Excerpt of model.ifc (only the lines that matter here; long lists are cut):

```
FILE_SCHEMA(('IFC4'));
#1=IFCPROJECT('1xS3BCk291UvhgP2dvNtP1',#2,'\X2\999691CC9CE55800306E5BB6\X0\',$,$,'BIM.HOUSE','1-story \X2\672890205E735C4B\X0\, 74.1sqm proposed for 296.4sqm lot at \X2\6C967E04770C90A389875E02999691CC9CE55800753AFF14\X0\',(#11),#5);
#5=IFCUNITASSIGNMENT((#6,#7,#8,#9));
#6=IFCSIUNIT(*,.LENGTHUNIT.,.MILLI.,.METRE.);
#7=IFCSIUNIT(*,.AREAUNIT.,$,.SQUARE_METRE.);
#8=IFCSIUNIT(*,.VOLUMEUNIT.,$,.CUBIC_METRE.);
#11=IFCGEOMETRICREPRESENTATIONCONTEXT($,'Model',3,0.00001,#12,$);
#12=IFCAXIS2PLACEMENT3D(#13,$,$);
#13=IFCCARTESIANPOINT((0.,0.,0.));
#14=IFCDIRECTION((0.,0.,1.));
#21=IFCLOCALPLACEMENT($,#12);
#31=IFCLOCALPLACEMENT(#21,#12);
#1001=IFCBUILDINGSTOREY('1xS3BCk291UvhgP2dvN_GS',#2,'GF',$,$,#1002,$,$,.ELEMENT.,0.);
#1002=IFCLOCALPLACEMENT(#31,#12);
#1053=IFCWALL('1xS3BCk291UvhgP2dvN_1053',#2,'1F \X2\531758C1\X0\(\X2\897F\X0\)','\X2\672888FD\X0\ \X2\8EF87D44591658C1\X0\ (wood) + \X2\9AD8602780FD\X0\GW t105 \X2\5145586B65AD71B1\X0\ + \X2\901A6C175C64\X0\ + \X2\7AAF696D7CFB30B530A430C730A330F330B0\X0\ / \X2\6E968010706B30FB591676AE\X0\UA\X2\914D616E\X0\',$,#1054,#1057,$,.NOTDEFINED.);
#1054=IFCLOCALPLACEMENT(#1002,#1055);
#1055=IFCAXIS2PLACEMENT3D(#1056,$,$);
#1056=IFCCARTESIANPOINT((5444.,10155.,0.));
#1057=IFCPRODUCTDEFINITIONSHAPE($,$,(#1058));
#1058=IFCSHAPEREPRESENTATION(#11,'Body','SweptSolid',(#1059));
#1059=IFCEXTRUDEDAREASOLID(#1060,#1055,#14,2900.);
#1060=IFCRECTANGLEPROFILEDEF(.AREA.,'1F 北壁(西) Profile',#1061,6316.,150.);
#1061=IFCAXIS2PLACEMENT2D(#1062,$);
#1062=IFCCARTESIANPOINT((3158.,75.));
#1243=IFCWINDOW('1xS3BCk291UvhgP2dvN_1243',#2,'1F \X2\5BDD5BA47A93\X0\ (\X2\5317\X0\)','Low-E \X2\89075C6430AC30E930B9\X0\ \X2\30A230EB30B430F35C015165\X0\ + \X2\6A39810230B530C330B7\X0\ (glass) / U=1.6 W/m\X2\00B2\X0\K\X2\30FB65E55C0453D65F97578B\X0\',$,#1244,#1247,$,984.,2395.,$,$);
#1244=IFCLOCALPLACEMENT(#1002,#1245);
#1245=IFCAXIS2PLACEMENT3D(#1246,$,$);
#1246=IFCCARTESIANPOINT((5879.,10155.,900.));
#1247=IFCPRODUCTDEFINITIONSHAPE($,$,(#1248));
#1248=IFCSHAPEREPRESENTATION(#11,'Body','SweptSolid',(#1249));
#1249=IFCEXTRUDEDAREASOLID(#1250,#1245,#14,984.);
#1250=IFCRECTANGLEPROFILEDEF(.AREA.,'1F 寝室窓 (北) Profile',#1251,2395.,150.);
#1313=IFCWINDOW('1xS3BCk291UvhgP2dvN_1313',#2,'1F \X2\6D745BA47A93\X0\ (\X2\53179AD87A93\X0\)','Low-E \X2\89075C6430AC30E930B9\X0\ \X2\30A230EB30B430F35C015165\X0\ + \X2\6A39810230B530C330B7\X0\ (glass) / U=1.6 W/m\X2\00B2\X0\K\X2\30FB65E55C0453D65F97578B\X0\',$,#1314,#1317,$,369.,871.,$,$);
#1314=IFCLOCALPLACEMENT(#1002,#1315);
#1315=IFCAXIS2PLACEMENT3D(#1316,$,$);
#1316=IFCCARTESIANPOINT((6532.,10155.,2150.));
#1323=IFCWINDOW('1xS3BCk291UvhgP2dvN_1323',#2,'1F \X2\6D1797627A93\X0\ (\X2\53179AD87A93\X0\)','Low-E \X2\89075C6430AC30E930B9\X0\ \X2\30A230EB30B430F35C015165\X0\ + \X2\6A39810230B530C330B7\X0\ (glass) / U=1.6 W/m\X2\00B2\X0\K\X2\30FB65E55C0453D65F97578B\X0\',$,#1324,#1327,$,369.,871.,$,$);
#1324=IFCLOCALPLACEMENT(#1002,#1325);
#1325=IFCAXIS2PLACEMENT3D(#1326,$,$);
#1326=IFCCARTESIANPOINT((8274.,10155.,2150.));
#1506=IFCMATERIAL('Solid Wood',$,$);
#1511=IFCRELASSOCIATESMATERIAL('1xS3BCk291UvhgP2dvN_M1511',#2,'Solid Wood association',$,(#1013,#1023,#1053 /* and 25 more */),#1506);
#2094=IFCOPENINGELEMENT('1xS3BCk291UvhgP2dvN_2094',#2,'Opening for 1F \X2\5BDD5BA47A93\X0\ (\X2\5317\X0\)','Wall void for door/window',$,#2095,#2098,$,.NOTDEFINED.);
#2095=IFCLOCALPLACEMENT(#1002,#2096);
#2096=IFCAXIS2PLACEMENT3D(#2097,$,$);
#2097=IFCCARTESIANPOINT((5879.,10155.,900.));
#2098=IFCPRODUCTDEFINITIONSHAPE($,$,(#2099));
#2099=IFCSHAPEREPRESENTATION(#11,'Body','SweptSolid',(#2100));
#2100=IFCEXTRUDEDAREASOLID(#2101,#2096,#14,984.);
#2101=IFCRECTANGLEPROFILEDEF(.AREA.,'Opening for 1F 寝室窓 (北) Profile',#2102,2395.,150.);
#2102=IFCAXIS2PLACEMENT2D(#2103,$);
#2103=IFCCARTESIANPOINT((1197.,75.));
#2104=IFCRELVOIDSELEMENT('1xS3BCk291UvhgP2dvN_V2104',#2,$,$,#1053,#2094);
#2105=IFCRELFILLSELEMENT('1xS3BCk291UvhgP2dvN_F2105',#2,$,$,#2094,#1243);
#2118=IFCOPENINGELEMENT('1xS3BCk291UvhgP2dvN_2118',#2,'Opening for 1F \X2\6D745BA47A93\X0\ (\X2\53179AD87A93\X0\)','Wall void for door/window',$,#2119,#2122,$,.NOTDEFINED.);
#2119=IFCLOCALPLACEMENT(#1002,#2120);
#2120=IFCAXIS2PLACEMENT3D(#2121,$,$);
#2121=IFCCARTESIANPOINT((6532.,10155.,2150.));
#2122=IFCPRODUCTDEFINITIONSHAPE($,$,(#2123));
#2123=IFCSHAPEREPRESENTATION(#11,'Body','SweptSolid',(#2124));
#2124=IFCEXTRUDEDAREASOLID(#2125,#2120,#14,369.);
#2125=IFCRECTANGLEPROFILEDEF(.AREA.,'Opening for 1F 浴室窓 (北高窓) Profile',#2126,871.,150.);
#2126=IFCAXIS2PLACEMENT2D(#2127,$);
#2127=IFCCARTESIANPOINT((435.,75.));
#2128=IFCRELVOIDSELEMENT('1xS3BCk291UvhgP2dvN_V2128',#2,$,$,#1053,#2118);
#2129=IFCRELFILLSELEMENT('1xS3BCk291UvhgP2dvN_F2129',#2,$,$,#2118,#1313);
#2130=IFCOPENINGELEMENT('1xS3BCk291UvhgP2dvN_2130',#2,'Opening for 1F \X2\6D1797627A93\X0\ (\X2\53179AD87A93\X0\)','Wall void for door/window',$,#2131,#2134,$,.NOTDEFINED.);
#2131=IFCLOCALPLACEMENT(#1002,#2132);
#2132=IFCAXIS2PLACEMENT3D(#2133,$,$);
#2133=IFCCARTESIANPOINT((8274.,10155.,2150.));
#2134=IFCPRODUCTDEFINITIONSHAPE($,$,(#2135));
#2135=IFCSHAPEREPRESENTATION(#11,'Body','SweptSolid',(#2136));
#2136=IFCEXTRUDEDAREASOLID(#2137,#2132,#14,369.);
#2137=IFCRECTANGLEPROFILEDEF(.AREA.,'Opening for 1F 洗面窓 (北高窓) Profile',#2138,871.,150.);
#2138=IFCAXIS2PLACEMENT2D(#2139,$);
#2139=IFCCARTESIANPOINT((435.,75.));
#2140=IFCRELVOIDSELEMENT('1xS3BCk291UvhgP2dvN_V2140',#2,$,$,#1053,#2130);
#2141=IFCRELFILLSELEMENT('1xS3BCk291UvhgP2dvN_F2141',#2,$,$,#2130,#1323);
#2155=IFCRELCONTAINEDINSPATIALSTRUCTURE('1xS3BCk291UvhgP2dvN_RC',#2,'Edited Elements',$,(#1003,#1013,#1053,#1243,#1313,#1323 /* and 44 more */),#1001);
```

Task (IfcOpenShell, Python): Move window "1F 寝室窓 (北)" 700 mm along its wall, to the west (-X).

```python
import ifcopenshell
import ifcopenshell.api.geometry
import ifcopenshell.util.placement
import ifcopenshell.util.unit

model = ifcopenshell.open("model.ifc")
unit_scale = ifcopenshell.util.unit.calculate_unit_scale(model)

window = model.by_guid("1xS3BCk291UvhgP2dvN_1243")
opening = window.FillsVoids[0].RelatingOpeningElement
wall = opening.VoidsElements[0].RelatingBuildingElement

wall_matrix = ifcopenshell.util.placement.get_local_placement(wall.ObjectPlacement)
shift = wall_matrix[:3, 0] * -0.7 / unit_scale
before = ifcopenshell.util.placement.get_local_placement(window.ObjectPlacement)[:3, 3].copy()

# The window is not placed relative to its opening, so move both.
for product in (opening, window):
    matrix = ifcopenshell.util.placement.get_local_placement(product.ObjectPlacement)
    matrix[:3, 3] += shift
    ifcopenshell.api.geometry.edit_object_placement(model, product=product, matrix=matrix, is_si=False)

after = ifcopenshell.util.placement.get_local_placement(window.ObjectPlacement)[:3, 3]
print("window moved by", (after - before).round(3) + 0.0)

model.write("model_rev.ifc")
```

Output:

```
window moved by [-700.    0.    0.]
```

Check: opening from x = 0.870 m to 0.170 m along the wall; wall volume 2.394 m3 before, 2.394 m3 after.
